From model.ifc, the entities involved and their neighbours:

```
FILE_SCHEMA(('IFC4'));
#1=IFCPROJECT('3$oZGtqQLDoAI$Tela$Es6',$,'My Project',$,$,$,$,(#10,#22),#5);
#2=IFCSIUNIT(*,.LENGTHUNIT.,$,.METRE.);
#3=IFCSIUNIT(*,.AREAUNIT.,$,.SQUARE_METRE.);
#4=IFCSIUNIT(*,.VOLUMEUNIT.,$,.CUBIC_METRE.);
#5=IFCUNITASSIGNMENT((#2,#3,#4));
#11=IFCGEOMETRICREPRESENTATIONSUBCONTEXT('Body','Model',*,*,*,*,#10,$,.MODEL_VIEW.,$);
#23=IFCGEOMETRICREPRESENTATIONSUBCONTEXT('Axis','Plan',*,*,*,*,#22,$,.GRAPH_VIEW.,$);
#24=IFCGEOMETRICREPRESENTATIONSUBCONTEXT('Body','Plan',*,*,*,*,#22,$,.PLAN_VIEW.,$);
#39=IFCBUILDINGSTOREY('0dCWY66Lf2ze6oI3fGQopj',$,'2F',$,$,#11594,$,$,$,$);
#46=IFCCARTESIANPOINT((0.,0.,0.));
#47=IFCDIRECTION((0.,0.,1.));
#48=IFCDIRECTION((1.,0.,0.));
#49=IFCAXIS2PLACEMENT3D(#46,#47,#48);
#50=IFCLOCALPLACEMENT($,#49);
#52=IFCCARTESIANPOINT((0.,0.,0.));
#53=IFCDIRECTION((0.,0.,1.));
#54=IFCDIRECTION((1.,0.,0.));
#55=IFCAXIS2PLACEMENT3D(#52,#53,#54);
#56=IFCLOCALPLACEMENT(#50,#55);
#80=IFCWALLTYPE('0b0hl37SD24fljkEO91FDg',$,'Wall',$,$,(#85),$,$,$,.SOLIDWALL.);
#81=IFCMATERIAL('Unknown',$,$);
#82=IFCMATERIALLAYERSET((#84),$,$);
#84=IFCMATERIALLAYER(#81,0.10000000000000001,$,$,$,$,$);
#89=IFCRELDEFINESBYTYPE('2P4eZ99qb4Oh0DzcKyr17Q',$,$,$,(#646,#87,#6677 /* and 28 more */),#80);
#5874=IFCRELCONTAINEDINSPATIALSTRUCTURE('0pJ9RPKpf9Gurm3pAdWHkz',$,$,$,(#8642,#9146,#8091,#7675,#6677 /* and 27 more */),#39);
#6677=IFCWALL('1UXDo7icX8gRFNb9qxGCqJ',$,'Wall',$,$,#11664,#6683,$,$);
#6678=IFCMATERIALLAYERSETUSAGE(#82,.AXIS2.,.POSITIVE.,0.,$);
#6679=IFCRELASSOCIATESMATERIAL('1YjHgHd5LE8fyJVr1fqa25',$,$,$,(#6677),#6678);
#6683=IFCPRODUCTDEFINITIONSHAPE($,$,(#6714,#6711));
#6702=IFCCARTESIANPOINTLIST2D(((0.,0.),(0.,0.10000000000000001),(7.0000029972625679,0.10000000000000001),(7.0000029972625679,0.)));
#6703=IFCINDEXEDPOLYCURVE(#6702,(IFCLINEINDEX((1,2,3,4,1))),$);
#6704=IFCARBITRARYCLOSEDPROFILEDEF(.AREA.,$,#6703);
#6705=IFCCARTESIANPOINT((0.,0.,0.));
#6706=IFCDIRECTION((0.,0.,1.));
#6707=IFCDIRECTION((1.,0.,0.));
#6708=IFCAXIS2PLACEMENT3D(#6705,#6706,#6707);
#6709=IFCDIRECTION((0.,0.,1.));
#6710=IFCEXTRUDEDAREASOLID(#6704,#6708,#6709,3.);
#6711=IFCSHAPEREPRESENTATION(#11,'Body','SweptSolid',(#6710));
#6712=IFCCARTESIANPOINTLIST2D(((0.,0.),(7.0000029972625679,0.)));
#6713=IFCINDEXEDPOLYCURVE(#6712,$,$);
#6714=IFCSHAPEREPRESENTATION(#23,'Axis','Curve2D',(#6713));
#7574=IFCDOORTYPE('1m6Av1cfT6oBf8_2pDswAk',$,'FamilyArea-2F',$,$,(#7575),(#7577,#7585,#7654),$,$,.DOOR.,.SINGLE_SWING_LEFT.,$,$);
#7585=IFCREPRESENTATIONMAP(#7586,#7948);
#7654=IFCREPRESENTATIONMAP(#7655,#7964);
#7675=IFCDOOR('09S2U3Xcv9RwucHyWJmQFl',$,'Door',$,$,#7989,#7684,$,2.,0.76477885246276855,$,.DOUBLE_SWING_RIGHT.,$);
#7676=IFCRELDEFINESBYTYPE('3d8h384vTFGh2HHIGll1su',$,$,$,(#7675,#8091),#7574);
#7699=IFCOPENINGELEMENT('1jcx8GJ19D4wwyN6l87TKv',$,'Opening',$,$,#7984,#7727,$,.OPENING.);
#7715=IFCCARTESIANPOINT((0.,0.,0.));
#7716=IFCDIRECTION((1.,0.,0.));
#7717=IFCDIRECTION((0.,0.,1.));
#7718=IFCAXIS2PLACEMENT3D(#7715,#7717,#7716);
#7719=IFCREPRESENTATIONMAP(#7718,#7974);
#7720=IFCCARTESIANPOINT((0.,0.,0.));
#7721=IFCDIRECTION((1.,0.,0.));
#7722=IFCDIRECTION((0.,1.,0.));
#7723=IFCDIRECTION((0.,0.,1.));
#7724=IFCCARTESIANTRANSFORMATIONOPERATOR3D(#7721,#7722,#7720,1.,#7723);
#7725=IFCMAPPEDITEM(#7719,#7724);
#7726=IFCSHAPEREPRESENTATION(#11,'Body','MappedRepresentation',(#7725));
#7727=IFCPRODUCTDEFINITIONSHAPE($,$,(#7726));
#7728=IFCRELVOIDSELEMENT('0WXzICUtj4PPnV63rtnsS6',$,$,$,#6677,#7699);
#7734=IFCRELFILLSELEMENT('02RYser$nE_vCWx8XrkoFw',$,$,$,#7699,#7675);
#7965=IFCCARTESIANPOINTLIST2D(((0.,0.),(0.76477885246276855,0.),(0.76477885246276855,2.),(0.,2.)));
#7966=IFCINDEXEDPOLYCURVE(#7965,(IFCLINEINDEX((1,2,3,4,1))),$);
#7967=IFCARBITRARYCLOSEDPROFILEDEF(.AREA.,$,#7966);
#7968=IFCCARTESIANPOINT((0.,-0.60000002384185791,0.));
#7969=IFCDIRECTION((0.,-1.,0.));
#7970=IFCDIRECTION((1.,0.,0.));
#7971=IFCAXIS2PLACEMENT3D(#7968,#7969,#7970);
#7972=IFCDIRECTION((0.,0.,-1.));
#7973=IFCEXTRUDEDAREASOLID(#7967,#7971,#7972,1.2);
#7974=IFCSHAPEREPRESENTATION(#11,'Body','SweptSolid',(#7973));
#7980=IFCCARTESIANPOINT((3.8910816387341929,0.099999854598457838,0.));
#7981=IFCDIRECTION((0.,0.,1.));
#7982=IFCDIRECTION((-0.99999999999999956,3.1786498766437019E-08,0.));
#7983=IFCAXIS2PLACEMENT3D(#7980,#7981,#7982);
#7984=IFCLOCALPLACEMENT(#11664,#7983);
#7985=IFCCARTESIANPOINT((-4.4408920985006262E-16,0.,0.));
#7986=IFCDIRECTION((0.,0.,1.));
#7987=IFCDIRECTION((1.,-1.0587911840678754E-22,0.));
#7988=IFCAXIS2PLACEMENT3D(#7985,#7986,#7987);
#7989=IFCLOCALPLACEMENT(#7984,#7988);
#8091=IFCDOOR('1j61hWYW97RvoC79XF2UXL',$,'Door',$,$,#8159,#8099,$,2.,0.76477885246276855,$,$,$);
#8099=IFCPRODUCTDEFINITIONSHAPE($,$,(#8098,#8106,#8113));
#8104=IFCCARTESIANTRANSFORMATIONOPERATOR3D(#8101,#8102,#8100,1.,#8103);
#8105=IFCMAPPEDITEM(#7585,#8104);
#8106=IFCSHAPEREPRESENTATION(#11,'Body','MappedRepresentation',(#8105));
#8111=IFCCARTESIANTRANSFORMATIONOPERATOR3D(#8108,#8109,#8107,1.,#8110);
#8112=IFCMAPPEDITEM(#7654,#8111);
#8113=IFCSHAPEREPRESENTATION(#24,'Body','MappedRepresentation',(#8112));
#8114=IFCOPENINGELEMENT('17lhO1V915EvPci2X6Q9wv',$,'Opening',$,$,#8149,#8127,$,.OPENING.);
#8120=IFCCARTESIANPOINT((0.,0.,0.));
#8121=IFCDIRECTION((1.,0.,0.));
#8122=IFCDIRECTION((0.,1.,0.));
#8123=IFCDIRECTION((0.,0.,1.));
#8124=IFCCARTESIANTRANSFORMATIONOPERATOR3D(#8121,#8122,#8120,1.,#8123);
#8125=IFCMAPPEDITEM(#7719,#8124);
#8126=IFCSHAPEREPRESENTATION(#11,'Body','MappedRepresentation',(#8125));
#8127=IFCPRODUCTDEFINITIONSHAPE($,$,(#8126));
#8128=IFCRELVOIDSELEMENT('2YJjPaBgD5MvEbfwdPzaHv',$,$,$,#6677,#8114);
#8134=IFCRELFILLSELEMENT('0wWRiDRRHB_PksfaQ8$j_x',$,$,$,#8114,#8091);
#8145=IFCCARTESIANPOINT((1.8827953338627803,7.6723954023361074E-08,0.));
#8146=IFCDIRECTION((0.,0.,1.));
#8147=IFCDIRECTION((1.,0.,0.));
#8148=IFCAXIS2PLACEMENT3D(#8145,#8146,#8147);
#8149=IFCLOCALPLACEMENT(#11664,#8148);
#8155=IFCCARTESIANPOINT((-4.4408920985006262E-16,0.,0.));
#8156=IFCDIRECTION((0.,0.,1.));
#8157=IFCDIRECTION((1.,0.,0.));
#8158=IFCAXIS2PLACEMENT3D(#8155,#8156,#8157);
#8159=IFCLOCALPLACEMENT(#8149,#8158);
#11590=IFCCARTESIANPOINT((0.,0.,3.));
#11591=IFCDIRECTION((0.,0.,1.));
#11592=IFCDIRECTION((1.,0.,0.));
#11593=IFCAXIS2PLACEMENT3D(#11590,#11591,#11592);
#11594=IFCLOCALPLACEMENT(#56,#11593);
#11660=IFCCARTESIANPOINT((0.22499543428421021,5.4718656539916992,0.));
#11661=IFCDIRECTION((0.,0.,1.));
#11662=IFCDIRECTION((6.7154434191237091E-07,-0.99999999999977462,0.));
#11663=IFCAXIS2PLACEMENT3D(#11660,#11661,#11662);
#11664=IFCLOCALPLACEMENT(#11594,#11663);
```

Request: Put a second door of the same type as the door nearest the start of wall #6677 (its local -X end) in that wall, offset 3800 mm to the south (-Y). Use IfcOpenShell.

```python
import ifcopenshell
import ifcopenshell.api.feature
import ifcopenshell.api.geometry
import ifcopenshell.api.root
import ifcopenshell.geom
import ifcopenshell.util.element
import ifcopenshell.util.placement
import ifcopenshell.util.shape
import ifcopenshell.util.unit

model = ifcopenshell.open("model.ifc")
unit_scale = ifcopenshell.util.unit.calculate_unit_scale(model)
settings = ifcopenshell.geom.settings()


def volume(element):
    """Net volume in cubic metres, openings subtracted."""
    shape = ifcopenshell.geom.create_shape(settings, element)
    return ifcopenshell.util.shape.get_volume(shape.geometry)


door = model.by_id(8091)
opening = door.FillsVoids[0].RelatingOpeningElement
wall = opening.VoidsElements[0].RelatingBuildingElement
before = volume(wall)
shift = ifcopenshell.util.placement.get_local_placement(wall.ObjectPlacement)[:3, 0] * 3.8 / unit_scale

# copy_class copies the void relationship, type, container and properties, but no geometry.
new_opening = ifcopenshell.api.root.copy_class(model, product=opening)
new_opening.Representation = ifcopenshell.util.element.copy_deep(
    model, opening.Representation, exclude=["IfcGeometricRepresentationContext", "IfcRepresentationMap"]
)
new_door = ifcopenshell.api.root.copy_class(model, product=door)
new_door.Representation = ifcopenshell.util.element.copy_deep(
    model, door.Representation, exclude=["IfcGeometricRepresentationContext", "IfcRepresentationMap"]
)
ifcopenshell.api.feature.add_filling(model, opening=new_opening, element=new_door)

for old, new in ((opening, new_opening), (door, new_door)):
    matrix = ifcopenshell.util.placement.get_local_placement(old.ObjectPlacement)
    matrix[:3, 3] += shift
    ifcopenshell.api.geometry.edit_object_placement(model, product=new, matrix=matrix, is_si=False)

after = volume(wall)

print(f"wall volume {before:.3f} -> {after:.3f} m3")

model.write("model_updated.ifc")
```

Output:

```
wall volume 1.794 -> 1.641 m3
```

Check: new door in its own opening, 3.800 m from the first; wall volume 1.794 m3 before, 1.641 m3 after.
